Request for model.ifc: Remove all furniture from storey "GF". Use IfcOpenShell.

First a look at what the model holds.

```python
import ifcopenshell
import ifcopenshell.util.element

model = ifcopenshell.open("model.ifc")
print(model.schema)
storey = next(s for s in model.by_type("IfcBuildingStorey") if s.Name == "GF")
furniture = [e for e in ifcopenshell.util.element.get_decomposition(storey) if e.is_a("IfcFurnishingElement")]
seen = {}
for e in furniture:
    element_type = ifcopenshell.util.element.get_type(e)
    name = element_type.Name if element_type not in (None, e) else None
    seen[name] = seen.get(name, 0) + 1
for name, count in sorted(seen.items(), key=str):
    print(count, "x", name)
```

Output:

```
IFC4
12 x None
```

```python
import ifcopenshell
import ifcopenshell.api.root
import ifcopenshell.util.element

model = ifcopenshell.open("model.ifc")

storey = next(s for s in model.by_type("IfcBuildingStorey") if s.Name == "GF")
furniture = [e for e in ifcopenshell.util.element.get_decomposition(storey) if e.is_a("IfcFurnishingElement")]

for e in furniture:
    ifcopenshell.api.root.remove_product(model, product=e)
print(len(furniture), "removed")

model.write("model-out.ifc")
```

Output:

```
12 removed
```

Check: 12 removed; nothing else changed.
